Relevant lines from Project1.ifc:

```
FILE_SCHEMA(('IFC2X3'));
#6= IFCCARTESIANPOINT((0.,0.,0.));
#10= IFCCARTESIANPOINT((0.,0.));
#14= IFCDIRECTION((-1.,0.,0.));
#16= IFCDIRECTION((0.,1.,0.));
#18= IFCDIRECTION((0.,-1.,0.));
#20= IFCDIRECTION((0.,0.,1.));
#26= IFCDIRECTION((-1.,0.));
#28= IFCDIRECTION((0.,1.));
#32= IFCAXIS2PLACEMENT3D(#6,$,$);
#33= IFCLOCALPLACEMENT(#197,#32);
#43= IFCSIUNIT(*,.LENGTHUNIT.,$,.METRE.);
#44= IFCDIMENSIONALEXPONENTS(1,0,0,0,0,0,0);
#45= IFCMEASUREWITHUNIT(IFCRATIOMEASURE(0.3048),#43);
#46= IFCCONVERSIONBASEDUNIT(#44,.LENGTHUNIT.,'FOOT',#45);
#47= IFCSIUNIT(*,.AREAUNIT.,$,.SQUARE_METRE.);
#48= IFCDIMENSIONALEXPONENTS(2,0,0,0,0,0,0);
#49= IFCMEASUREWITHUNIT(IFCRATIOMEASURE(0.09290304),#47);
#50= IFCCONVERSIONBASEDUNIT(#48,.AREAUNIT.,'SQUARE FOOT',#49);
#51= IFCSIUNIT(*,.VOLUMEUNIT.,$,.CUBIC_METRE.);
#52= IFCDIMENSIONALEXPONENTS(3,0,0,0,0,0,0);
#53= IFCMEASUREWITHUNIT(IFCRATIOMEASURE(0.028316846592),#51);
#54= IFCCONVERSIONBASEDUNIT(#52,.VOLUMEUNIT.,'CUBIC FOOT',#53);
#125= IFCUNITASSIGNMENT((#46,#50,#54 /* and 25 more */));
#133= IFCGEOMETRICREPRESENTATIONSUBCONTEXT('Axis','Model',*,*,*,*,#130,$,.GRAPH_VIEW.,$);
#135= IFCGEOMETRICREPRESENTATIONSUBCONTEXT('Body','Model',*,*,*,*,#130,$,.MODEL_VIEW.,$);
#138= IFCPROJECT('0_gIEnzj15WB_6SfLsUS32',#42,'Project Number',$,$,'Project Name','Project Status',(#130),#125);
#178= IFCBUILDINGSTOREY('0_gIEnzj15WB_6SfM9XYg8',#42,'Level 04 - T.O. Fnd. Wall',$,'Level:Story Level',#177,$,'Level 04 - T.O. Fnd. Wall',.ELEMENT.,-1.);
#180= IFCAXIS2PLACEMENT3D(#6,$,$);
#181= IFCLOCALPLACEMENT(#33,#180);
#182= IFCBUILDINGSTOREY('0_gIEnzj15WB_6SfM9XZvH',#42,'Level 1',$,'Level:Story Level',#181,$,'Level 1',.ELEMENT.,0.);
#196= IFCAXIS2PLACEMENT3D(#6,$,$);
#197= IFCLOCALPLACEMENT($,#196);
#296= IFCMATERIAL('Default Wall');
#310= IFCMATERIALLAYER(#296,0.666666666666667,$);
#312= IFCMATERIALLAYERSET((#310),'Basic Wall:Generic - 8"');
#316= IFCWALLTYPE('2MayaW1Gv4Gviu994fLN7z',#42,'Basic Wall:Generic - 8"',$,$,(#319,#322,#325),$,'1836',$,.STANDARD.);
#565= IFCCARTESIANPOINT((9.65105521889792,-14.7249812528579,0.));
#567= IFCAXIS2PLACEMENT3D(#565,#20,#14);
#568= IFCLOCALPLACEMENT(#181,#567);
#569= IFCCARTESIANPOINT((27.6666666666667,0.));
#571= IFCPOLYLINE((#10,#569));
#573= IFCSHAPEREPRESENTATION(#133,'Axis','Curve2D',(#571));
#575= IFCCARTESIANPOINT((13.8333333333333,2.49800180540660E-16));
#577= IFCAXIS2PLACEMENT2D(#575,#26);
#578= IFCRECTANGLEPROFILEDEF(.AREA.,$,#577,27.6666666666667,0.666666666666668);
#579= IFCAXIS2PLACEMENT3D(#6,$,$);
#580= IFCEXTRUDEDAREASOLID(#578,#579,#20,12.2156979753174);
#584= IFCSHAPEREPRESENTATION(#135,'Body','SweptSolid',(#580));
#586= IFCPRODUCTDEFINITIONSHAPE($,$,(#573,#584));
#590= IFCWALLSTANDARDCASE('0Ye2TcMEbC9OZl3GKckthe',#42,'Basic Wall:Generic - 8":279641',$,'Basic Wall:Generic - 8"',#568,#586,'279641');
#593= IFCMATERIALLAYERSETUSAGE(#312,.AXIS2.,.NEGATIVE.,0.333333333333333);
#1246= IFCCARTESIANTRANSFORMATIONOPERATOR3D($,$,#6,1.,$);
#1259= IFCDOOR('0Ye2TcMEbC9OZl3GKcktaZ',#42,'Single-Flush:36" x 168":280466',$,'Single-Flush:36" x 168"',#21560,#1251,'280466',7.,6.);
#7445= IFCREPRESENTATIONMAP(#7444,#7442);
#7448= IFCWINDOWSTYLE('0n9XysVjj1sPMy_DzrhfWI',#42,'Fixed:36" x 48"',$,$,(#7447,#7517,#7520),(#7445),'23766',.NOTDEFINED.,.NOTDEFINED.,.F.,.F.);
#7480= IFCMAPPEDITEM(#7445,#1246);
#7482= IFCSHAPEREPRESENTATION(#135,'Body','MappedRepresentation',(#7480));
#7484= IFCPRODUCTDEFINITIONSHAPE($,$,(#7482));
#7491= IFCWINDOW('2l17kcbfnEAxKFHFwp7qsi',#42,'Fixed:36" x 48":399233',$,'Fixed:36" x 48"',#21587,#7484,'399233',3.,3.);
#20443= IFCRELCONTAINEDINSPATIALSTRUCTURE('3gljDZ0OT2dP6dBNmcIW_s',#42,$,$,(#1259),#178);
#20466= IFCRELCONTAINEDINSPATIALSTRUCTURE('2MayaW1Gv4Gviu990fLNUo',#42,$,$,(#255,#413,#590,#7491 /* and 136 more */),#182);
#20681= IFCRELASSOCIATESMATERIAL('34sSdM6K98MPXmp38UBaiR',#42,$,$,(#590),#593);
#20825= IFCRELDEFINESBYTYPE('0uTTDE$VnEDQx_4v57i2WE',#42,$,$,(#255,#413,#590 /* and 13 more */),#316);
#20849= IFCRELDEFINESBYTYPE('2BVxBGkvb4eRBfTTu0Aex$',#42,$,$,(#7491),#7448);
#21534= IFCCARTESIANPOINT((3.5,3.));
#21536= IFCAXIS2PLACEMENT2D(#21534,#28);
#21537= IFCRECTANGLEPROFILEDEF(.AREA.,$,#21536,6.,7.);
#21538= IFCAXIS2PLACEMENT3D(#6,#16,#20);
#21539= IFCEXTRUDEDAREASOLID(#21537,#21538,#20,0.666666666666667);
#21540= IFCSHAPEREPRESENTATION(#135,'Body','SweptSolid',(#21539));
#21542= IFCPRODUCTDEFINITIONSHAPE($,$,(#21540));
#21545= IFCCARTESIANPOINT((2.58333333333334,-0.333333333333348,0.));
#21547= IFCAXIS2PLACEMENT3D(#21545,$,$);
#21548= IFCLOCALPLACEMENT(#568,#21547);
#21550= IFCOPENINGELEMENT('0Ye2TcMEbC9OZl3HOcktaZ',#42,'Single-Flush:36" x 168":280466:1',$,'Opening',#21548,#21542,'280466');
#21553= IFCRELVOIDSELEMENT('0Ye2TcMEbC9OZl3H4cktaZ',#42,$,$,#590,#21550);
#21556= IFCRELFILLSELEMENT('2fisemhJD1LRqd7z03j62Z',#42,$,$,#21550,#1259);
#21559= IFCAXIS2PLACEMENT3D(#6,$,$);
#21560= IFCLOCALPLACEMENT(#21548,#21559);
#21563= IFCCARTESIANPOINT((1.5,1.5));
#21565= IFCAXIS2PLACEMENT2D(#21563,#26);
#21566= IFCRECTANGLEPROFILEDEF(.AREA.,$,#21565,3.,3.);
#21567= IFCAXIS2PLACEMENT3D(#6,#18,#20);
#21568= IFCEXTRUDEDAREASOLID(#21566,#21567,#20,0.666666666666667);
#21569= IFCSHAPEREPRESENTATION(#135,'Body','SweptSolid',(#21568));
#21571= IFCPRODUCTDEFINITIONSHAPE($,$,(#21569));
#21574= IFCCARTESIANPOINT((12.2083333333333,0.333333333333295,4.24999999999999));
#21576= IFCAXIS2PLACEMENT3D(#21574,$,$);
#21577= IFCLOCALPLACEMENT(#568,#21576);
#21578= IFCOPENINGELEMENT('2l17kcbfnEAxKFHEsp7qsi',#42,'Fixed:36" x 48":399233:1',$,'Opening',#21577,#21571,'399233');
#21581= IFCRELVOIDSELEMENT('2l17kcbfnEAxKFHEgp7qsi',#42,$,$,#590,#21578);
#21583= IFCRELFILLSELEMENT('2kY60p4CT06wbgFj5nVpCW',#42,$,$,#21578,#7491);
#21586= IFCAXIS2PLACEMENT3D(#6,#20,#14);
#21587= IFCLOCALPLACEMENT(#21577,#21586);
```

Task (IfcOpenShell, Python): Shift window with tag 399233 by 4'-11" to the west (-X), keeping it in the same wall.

```python
import ifcopenshell
import ifcopenshell.api.geometry
import ifcopenshell.util.placement
import ifcopenshell.util.unit

model = ifcopenshell.open("Project1.ifc")
unit_scale = ifcopenshell.util.unit.calculate_unit_scale(model)

window = model.by_guid("2l17kcbfnEAxKFHFwp7qsi")
opening = window.FillsVoids[0].RelatingOpeningElement
wall = opening.VoidsElements[0].RelatingBuildingElement

wall_matrix = ifcopenshell.util.placement.get_local_placement(wall.ObjectPlacement)
shift = wall_matrix[:3, 0] * 59 * 0.0254 / unit_scale
before = ifcopenshell.util.placement.get_local_placement(window.ObjectPlacement)[:3, 3].copy()

# The window is placed relative to its opening, so it follows when the opening moves.
matrix = ifcopenshell.util.placement.get_local_placement(opening.ObjectPlacement)
matrix[:3, 3] += shift
ifcopenshell.api.geometry.edit_object_placement(
    model, product=opening, matrix=matrix, is_si=False, should_transform_children=True
)

after = ifcopenshell.util.placement.get_local_placement(window.ObjectPlacement)[:3, 3]
print("window moved by", (after - before).round(3) + 0.0)

model.write("Project1_updated.ifc")
```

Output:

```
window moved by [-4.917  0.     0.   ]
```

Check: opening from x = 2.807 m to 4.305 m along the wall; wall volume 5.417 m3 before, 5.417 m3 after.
